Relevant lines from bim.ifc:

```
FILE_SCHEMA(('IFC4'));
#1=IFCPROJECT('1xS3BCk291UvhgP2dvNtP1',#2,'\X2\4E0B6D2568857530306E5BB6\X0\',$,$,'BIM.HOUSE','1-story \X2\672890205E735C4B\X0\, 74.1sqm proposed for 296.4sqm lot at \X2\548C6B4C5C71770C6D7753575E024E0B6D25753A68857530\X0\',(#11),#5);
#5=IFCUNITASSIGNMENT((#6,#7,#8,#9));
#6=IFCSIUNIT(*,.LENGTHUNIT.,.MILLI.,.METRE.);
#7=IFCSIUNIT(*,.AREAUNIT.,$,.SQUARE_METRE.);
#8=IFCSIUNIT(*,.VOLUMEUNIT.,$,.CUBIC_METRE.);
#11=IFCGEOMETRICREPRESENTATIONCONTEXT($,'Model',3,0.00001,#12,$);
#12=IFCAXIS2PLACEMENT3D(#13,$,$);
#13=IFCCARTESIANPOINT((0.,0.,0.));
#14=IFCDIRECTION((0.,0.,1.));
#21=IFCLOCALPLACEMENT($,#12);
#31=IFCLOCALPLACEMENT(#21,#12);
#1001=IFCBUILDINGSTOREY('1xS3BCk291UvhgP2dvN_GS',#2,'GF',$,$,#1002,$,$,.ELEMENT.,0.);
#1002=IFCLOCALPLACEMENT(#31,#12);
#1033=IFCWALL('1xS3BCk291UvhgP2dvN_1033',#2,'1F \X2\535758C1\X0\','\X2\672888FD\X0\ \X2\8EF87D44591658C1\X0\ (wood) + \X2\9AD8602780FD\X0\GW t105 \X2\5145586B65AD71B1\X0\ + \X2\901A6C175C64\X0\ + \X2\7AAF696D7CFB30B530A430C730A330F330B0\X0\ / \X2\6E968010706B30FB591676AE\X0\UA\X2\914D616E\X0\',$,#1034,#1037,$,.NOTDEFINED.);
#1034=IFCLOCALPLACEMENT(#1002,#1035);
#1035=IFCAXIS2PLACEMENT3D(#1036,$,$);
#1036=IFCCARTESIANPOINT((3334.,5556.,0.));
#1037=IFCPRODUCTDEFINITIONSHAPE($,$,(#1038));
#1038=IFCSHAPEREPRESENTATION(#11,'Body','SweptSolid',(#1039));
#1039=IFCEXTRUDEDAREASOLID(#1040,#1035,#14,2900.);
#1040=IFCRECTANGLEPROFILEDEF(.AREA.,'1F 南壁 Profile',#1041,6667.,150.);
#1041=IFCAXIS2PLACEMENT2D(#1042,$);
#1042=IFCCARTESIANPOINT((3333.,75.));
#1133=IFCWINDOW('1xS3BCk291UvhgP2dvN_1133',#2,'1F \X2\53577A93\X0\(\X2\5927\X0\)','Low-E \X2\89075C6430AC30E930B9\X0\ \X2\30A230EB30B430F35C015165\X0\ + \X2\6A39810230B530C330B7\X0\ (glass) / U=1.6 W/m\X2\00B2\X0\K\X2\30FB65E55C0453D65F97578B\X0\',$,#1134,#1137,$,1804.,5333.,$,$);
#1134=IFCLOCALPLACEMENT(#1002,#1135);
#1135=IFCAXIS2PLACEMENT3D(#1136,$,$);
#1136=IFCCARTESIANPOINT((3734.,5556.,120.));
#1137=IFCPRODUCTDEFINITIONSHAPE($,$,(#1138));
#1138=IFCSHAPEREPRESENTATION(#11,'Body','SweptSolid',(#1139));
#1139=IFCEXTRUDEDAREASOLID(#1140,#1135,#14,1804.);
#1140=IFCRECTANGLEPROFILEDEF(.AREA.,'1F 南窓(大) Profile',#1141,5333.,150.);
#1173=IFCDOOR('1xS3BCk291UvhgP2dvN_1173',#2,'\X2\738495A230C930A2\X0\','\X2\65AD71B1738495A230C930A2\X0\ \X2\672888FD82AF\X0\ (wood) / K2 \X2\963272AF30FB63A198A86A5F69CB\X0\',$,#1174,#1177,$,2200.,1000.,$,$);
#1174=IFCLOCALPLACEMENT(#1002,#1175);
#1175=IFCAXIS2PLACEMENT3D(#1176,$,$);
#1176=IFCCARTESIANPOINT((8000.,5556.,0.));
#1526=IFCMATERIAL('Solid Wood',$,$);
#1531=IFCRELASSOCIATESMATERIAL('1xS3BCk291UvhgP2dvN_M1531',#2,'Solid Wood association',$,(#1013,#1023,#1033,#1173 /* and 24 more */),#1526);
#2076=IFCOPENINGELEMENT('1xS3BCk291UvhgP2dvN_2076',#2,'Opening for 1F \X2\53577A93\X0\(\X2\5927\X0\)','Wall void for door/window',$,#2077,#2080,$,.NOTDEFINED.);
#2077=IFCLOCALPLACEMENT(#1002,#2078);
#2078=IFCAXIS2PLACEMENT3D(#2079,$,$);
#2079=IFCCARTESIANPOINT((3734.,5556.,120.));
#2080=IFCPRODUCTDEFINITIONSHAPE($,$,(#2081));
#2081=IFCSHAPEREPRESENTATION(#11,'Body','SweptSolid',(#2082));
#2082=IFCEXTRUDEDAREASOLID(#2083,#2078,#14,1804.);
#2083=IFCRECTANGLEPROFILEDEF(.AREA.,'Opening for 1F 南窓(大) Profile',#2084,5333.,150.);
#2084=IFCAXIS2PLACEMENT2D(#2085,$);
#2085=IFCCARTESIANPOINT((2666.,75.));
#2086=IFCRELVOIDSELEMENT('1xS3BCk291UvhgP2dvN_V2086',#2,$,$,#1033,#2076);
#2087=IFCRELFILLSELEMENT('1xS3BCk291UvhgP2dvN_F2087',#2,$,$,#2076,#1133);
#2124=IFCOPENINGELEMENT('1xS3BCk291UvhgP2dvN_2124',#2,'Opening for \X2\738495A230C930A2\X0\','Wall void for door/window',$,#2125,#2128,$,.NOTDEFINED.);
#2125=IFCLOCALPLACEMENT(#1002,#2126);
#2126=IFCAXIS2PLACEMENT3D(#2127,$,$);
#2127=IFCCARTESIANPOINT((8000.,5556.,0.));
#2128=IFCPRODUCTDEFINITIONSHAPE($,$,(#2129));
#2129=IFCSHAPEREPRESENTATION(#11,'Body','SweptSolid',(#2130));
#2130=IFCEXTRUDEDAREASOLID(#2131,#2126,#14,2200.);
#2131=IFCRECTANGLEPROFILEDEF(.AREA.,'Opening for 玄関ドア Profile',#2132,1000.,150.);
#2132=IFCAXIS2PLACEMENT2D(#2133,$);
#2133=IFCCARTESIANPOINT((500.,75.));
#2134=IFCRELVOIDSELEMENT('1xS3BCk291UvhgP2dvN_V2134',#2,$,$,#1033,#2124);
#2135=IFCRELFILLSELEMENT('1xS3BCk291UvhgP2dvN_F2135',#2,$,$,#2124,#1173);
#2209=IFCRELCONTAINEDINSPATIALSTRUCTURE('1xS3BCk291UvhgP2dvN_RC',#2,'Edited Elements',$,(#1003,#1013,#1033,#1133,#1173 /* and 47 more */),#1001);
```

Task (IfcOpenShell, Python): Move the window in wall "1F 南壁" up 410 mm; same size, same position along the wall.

```python
import numpy as np
import ifcopenshell
import ifcopenshell.api.geometry
import ifcopenshell.util.placement
import ifcopenshell.util.unit

model = ifcopenshell.open("bim.ifc")
unit_scale = ifcopenshell.util.unit.calculate_unit_scale(model)

window = model.by_guid("1xS3BCk291UvhgP2dvN_1133")
opening = window.FillsVoids[0].RelatingOpeningElement
dz = 0.41 / unit_scale

shift = np.array([0.0, 0.0, dz])
# The window is not placed relative to its opening, so move both.
for product in (opening, window):
    matrix = ifcopenshell.util.placement.get_local_placement(product.ObjectPlacement)
    matrix[:3, 3] += shift
    ifcopenshell.api.geometry.edit_object_placement(model, product=product, matrix=matrix, is_si=False)

print(f"moved by {dz * unit_scale:+.3f} m")

model.write("bim_updated.ifc")
```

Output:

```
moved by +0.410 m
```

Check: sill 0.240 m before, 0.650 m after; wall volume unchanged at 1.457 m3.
